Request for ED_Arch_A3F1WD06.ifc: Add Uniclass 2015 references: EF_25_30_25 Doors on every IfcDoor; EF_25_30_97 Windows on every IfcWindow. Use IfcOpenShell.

First a look at what the model holds.

```python
import ifcopenshell

model = ifcopenshell.open("ED_Arch_A3F1WD06.ifc")
print(model.schema)
print("classifications:", [c.Name for c in model.by_type("IfcClassification")])
for ifc_class in ("IfcDoor", "IfcRoof", "IfcStair", "IfcWall", "IfcWindow"):
    print(ifc_class, len(model.by_type(ifc_class)))
```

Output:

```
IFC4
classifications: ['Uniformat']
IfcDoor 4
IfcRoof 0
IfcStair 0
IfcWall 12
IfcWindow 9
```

```python
import ifcopenshell
import ifcopenshell.api.classification

model = ifcopenshell.open("ED_Arch_A3F1WD06.ifc")

system = ifcopenshell.api.classification.add_classification(model, classification="Uniclass 2015")

codes = {
    "IfcDoor": ("EF_25_30_25", "Doors"),
    "IfcWindow": ("EF_25_30_97", "Windows"),
}
for ifc_class, (code, name) in codes.items():
    products = model.by_type(ifc_class)
    ifcopenshell.api.classification.add_reference(
        model, products=products, classification=system, identification=code, name=name
    )
    print(code, len(products))

model.write("ED_Arch_A3F1WD06_rev.ifc")
```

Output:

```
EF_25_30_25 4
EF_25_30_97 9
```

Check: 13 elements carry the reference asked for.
